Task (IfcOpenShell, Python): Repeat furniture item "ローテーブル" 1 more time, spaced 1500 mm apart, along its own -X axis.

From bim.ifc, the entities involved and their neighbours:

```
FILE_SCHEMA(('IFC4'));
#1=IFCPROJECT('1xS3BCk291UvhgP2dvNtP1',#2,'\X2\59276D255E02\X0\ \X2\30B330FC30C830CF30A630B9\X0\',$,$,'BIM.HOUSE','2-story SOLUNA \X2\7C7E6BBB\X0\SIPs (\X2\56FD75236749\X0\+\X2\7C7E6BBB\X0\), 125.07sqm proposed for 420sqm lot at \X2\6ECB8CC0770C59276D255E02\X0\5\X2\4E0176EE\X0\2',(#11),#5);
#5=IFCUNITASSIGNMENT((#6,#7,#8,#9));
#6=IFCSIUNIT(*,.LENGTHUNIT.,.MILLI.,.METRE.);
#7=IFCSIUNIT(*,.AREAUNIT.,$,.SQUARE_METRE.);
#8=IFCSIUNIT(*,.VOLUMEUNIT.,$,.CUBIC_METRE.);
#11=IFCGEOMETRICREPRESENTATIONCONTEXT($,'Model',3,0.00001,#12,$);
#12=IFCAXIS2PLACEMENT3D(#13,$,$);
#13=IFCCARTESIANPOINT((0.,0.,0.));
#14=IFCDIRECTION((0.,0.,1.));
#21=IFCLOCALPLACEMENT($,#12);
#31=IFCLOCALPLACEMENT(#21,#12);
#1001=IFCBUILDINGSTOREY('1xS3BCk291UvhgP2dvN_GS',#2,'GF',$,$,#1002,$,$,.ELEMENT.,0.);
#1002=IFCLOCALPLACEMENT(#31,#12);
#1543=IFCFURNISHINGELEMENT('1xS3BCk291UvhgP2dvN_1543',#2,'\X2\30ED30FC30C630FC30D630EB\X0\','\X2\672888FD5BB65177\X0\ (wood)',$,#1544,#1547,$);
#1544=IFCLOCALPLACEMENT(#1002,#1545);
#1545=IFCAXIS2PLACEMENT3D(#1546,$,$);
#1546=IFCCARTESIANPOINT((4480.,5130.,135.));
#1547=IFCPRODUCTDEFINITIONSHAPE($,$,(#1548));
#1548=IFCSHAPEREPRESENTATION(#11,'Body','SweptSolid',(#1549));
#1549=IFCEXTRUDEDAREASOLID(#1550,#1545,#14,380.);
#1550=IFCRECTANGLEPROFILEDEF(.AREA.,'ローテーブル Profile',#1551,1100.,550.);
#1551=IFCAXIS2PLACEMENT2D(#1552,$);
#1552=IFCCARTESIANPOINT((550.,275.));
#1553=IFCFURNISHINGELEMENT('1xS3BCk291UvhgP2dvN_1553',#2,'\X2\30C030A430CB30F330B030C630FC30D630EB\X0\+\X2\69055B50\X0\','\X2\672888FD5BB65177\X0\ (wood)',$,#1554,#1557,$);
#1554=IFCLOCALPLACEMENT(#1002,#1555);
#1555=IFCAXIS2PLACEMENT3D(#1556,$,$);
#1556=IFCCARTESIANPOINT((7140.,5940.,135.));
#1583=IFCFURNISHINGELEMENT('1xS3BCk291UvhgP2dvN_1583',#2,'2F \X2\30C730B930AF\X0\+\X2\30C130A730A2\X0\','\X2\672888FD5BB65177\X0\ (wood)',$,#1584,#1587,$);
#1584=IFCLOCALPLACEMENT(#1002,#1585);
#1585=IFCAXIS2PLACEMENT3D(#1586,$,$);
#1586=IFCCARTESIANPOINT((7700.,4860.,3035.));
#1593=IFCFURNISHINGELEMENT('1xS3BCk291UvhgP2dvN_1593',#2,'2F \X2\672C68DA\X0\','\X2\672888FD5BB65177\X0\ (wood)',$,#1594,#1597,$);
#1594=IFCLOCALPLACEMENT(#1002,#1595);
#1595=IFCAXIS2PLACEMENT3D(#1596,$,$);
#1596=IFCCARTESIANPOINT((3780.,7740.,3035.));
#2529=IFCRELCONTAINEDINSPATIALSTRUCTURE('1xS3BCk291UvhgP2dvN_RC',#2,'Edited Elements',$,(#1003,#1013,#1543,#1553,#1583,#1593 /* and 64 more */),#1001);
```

```python
import ifcopenshell
import ifcopenshell.api.geometry
import ifcopenshell.api.root
import ifcopenshell.util.element
import ifcopenshell.util.placement
import ifcopenshell.util.unit

model = ifcopenshell.open("bim.ifc")
unit_scale = ifcopenshell.util.unit.calculate_unit_scale(model)


def reuse_history(source, copy):
    """copy_class also copies each property set's owner history, people and application; keep the originals."""
    for rel in copy.IsDefinedBy:
        if rel.is_a("IfcRelDefinesByProperties") and (history := rel.RelatingPropertyDefinition.OwnerHistory):
            rel.RelatingPropertyDefinition.OwnerHistory = source.OwnerHistory
            ifcopenshell.util.element.remove_deep2(model, history)


source = model.by_guid("1xS3BCk291UvhgP2dvN_1543")
base = ifcopenshell.util.placement.get_local_placement(source.ObjectPlacement)
step = -base[:3, 0] * 1.5 / unit_scale

for i in range(1, 2):
    copy = ifcopenshell.api.root.copy_class(model, product=source)
    copy.Representation = ifcopenshell.util.element.copy_deep(
        model, source.Representation, exclude=["IfcGeometricRepresentationContext", "IfcRepresentationMap"]
    )
    reuse_history(source, copy)
    matrix = base.copy()
    matrix[:3, 3] += i * step
    print("added at", matrix[:3, 3].round(3) + 0.0)
    ifcopenshell.api.geometry.edit_object_placement(model, product=copy, matrix=matrix, is_si=False)

model.write("bim_rev.ifc")
```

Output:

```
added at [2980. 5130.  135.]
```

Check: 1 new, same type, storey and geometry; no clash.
